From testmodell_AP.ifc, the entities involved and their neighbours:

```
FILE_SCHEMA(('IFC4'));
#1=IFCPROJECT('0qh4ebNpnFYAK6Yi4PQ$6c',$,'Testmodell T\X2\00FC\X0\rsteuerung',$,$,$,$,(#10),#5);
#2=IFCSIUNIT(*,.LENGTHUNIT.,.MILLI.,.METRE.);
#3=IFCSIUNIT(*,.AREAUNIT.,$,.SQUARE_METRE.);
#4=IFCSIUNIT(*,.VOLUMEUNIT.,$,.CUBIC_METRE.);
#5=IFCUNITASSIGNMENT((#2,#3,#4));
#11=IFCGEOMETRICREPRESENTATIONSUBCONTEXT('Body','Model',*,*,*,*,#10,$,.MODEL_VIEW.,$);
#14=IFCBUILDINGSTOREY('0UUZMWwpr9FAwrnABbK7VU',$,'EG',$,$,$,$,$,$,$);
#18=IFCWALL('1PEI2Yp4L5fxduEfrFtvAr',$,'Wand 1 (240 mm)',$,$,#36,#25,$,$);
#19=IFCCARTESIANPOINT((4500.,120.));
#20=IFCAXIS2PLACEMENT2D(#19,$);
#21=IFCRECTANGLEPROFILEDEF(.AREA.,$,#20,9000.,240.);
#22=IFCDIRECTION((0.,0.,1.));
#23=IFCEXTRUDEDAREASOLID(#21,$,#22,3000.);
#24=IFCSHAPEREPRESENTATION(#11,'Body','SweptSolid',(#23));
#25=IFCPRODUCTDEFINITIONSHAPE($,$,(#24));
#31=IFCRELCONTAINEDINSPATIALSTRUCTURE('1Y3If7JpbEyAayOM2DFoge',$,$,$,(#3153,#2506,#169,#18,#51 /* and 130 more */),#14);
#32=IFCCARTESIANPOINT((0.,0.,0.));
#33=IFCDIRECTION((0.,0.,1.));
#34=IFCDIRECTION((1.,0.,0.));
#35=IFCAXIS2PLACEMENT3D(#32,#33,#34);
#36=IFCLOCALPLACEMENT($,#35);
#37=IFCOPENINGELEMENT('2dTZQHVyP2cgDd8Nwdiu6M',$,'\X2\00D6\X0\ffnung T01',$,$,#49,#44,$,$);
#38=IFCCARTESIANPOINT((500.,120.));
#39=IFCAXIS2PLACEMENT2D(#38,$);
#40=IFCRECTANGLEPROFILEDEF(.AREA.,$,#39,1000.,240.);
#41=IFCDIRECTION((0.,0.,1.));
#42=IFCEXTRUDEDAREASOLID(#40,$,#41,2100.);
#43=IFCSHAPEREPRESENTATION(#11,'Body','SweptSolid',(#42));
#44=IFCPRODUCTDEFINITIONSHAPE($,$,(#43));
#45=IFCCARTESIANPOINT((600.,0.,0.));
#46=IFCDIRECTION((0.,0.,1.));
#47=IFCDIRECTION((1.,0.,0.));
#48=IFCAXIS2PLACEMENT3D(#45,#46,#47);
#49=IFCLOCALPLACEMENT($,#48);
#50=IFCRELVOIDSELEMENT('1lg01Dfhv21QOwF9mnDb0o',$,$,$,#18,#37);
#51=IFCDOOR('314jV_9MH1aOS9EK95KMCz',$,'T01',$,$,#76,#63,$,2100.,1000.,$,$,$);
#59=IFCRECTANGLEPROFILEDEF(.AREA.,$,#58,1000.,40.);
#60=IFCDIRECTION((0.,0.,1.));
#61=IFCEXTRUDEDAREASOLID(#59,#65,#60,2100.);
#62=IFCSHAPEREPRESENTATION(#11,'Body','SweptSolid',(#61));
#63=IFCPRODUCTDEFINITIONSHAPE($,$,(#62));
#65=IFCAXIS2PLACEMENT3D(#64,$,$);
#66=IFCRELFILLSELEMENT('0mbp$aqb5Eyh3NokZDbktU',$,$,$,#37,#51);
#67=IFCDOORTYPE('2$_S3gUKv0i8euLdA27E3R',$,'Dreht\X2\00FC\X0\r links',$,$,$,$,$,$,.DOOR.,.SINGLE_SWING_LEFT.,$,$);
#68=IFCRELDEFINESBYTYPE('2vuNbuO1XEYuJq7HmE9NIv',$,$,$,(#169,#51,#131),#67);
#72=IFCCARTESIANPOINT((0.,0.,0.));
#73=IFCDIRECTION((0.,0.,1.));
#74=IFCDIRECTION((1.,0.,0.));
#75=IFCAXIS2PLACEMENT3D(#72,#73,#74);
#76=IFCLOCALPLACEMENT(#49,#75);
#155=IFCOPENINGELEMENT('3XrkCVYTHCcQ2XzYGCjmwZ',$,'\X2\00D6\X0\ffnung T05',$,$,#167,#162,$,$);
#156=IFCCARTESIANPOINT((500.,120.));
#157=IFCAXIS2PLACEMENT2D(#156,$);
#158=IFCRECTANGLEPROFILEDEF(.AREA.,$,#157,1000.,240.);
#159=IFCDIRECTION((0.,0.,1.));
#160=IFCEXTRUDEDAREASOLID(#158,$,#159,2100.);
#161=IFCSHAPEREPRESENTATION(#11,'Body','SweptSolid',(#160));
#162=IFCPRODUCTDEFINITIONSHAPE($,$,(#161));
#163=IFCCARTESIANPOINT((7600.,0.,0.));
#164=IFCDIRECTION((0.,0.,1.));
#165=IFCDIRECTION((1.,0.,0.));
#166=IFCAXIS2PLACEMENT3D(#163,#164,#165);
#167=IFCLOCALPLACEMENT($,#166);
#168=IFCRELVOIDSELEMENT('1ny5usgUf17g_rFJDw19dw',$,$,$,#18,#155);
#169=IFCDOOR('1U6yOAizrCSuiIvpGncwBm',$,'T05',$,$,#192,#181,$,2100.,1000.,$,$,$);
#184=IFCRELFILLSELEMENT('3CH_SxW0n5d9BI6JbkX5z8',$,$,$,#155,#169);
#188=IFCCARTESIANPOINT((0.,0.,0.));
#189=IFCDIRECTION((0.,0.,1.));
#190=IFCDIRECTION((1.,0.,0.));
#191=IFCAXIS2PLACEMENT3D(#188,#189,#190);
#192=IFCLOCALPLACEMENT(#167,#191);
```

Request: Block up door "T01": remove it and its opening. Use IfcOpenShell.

```python
import ifcopenshell
import ifcopenshell.api.feature
import ifcopenshell.api.root
import ifcopenshell.geom
import ifcopenshell.util.shape

model = ifcopenshell.open("testmodell_AP.ifc")
settings = ifcopenshell.geom.settings()


def volume(element):
    """Net volume in cubic metres, openings subtracted."""
    shape = ifcopenshell.geom.create_shape(settings, element)
    return ifcopenshell.util.shape.get_volume(shape.geometry)


door = model.by_guid("314jV_9MH1aOS9EK95KMCz")
opening = door.FillsVoids[0].RelatingOpeningElement
wall = opening.VoidsElements[0].RelatingBuildingElement
before = volume(wall)

ifcopenshell.api.root.remove_product(model, product=door)
ifcopenshell.api.feature.remove_feature(model, feature=opening)

after = volume(wall)

print(f"wall volume {before:.3f} -> {after:.3f} m3")

model.write("testmodell_AP_edited.ifc")
```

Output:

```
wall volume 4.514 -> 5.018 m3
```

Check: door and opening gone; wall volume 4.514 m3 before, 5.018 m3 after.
